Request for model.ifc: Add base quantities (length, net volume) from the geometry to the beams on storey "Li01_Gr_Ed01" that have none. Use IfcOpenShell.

First a look at what the model holds.

```python
import ifcopenshell
import ifcopenshell.util.element
import ifcopenshell.util.unit

model = ifcopenshell.open("model.ifc")
print(model.schema)
for unit_type in ("LENGTHUNIT", "AREAUNIT", "VOLUMEUNIT"):
    print(unit_type, ifcopenshell.util.unit.calculate_unit_scale(model, unit_type))
storey = next(s for s in model.by_type("IfcBuildingStorey") if s.Name == "Li01_Gr_Ed01")
beams = [e for e in ifcopenshell.util.element.get_decomposition(storey) if e.is_a("IfcBeam")]
for e in sorted(beams, key=lambda e: e.id()):
    print(e.id(), e.is_a(), e.Name, list(ifcopenshell.util.element.get_psets(e, qtos_only=True)), sep=" | ")
```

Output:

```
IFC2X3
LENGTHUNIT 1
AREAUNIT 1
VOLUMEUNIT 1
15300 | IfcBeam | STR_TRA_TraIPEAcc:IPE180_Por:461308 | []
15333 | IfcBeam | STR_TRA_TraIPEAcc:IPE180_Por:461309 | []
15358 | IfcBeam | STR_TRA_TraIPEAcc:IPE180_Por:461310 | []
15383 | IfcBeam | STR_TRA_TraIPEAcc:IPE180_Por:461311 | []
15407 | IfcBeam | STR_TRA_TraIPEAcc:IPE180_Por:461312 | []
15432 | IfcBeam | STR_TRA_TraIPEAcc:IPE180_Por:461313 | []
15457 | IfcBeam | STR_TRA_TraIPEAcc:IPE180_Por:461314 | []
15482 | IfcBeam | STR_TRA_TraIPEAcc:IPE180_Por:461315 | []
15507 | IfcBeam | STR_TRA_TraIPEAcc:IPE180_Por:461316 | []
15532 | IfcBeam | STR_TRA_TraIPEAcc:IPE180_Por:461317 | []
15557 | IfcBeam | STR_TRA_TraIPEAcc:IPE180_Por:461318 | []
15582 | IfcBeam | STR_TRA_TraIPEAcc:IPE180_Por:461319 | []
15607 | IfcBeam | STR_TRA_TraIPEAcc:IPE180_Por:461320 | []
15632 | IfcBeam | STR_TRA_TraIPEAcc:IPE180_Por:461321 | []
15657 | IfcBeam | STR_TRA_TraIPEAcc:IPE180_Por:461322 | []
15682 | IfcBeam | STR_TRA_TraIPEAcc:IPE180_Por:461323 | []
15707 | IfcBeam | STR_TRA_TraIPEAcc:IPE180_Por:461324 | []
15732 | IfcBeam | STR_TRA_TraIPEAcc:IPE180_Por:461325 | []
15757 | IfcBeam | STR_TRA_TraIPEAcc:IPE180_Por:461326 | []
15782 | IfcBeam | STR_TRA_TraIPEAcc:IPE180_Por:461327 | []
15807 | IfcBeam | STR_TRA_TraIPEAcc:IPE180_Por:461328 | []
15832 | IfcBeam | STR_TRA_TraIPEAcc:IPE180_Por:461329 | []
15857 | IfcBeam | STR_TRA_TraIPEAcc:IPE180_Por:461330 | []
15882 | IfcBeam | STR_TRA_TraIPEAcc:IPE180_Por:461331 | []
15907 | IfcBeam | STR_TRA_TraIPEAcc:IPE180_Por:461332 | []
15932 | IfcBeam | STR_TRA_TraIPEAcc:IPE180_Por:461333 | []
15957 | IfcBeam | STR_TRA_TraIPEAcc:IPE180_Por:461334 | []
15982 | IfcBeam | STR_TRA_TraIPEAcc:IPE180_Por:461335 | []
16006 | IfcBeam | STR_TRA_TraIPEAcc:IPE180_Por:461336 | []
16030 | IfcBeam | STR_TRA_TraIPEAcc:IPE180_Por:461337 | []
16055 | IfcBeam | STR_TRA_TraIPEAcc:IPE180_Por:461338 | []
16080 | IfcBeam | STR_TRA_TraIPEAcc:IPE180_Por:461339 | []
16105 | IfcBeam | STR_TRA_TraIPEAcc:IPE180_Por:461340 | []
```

```python
import ifcopenshell
import ifcopenshell.api.pset
import ifcopenshell.geom
import ifcopenshell.util.element
import ifcopenshell.util.shape
import ifcopenshell.util.unit

model = ifcopenshell.open("model.ifc")
unit_scale = ifcopenshell.util.unit.calculate_unit_scale(model)
volume_scale = ifcopenshell.util.unit.calculate_unit_scale(model, "VOLUMEUNIT")
settings = ifcopenshell.geom.settings()

storey = next(s for s in model.by_type("IfcBuildingStorey") if s.Name == "Li01_Gr_Ed01")
beams = [e for e in ifcopenshell.util.element.get_decomposition(storey) if e.is_a("IfcBeam")]

for e in sorted(beams, key=lambda e: e.id()):
    if ifcopenshell.util.element.get_psets(e, qtos_only=True, should_inherit=False):
        continue
    # Geometry comes back in metres, in the element's own axes.
    shape = ifcopenshell.geom.create_shape(settings, e)
    values = {
        "Length": ifcopenshell.util.shape.get_max_xyz(shape.geometry) / unit_scale,
        "NetVolume": ifcopenshell.util.shape.get_volume(shape.geometry) / volume_scale,
    }
    qto = ifcopenshell.api.pset.add_qto(model, product=e, name="BaseQuantities")
    ifcopenshell.api.pset.edit_qto(model, qto=qto, properties=values)
    print(e.id(), {k: round(v, 3) for k, v in values.items()})

model.write("model_rev.ifc")
```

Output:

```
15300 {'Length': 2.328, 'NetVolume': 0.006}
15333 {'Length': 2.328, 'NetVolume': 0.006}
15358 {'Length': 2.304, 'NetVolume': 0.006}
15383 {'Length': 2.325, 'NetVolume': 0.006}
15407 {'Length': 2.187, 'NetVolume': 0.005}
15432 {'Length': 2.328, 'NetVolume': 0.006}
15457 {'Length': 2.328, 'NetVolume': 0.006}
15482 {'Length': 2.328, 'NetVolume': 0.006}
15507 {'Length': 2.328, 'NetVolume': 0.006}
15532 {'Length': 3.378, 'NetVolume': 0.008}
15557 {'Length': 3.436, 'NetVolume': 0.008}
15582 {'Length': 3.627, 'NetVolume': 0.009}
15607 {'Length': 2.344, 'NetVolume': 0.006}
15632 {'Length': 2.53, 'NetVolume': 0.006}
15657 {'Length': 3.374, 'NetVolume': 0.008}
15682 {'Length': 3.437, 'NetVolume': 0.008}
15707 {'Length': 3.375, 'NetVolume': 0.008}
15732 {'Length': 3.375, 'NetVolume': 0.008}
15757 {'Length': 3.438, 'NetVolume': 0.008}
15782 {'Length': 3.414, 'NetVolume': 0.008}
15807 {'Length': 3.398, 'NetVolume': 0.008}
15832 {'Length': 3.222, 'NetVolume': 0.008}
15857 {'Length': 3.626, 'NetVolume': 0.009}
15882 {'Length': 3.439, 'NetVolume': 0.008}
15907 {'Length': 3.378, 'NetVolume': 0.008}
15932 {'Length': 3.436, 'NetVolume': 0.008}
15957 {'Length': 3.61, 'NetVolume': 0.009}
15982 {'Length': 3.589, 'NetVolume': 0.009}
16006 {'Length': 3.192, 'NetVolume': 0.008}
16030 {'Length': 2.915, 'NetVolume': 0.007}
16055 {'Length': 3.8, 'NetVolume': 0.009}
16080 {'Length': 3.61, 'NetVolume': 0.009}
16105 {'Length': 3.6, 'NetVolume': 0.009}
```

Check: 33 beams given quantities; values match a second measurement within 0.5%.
